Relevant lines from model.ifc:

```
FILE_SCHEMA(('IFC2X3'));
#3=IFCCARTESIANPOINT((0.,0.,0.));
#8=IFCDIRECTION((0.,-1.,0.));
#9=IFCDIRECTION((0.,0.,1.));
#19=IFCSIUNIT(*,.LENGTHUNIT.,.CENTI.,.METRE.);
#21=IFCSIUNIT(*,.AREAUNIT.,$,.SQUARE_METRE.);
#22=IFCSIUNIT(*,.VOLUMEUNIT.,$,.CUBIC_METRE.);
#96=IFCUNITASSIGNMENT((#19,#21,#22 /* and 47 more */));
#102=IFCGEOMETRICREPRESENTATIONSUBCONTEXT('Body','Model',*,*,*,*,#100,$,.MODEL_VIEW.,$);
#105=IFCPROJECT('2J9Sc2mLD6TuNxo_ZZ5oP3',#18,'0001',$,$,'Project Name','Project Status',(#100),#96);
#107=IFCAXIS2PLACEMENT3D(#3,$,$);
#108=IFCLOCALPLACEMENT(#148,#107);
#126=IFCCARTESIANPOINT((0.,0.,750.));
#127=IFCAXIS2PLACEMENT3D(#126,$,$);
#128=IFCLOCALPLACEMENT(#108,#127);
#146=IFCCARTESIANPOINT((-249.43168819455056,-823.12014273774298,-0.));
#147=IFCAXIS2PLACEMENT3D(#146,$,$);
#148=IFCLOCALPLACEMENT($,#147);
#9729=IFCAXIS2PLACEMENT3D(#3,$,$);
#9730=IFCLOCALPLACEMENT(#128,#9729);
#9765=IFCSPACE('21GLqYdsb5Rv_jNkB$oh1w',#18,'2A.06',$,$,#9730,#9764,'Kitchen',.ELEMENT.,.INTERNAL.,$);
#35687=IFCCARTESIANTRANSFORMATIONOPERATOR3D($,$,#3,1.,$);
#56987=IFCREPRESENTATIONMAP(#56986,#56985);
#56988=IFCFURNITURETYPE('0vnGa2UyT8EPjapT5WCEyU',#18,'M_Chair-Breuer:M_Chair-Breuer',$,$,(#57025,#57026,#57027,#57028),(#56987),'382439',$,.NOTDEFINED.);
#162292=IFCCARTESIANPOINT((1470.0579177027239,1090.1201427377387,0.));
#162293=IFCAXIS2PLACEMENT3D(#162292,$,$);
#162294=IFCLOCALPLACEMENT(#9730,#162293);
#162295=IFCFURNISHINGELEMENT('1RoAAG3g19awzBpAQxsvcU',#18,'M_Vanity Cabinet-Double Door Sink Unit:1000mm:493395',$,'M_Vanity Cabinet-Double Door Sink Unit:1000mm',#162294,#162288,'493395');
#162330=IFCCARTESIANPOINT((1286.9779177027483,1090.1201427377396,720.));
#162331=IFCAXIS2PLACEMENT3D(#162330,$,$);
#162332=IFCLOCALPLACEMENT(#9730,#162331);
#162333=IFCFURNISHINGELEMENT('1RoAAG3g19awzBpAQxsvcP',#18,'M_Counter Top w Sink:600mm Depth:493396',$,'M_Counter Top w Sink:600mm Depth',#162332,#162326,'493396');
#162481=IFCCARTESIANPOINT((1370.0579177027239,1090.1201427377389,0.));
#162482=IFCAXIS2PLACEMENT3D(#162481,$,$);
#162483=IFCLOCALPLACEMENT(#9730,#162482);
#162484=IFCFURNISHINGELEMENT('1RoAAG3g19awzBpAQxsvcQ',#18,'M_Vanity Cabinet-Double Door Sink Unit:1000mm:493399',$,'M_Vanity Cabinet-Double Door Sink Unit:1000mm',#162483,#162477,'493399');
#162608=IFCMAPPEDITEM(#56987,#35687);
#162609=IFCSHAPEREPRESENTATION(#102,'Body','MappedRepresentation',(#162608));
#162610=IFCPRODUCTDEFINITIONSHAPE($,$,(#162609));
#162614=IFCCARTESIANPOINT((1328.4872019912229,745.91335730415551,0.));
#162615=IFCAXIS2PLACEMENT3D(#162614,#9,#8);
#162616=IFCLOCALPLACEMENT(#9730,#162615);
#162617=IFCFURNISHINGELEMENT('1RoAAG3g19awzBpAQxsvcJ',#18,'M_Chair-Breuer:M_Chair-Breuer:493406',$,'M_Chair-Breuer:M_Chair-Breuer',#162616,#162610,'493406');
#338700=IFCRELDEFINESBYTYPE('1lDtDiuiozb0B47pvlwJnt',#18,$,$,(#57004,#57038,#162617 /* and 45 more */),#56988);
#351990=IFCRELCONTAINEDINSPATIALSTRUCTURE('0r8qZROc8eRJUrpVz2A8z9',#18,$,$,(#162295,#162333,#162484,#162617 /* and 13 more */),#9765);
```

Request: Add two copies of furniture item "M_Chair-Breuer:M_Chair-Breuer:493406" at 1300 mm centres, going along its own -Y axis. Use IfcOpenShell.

```python
import ifcopenshell
import ifcopenshell.api.geometry
import ifcopenshell.api.root
import ifcopenshell.util.element
import ifcopenshell.util.placement
import ifcopenshell.util.unit

model = ifcopenshell.open("model.ifc")
unit_scale = ifcopenshell.util.unit.calculate_unit_scale(model)


def reuse_history(source, copy):
    """copy_class also copies each property set's owner history, people and application; keep the originals."""
    for rel in copy.IsDefinedBy:
        if rel.is_a("IfcRelDefinesByProperties") and (history := rel.RelatingPropertyDefinition.OwnerHistory):
            rel.RelatingPropertyDefinition.OwnerHistory = source.OwnerHistory
            ifcopenshell.util.element.remove_deep2(model, history)


source = model.by_guid("1RoAAG3g19awzBpAQxsvcJ")
base = ifcopenshell.util.placement.get_local_placement(source.ObjectPlacement)
step = -base[:3, 1] * 1.3 / unit_scale

for i in range(1, 3):
    copy = ifcopenshell.api.root.copy_class(model, product=source)
    copy.Representation = ifcopenshell.util.element.copy_deep(
        model, source.Representation, exclude=["IfcGeometricRepresentationContext", "IfcRepresentationMap"]
    )
    copy.Name = "M_Chair-Breuer:M_Chair-Breuer"
    copy.Tag = None
    reuse_history(source, copy)
    matrix = base.copy()
    matrix[:3, 3] += i * step
    print("added at", matrix[:3, 3].round(3) + 0.0)
    ifcopenshell.api.geometry.edit_object_placement(model, product=copy, matrix=matrix, is_si=False)

model.write("model_edited.ifc")
```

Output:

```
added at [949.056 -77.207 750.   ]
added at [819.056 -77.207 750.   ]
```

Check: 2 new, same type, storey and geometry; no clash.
